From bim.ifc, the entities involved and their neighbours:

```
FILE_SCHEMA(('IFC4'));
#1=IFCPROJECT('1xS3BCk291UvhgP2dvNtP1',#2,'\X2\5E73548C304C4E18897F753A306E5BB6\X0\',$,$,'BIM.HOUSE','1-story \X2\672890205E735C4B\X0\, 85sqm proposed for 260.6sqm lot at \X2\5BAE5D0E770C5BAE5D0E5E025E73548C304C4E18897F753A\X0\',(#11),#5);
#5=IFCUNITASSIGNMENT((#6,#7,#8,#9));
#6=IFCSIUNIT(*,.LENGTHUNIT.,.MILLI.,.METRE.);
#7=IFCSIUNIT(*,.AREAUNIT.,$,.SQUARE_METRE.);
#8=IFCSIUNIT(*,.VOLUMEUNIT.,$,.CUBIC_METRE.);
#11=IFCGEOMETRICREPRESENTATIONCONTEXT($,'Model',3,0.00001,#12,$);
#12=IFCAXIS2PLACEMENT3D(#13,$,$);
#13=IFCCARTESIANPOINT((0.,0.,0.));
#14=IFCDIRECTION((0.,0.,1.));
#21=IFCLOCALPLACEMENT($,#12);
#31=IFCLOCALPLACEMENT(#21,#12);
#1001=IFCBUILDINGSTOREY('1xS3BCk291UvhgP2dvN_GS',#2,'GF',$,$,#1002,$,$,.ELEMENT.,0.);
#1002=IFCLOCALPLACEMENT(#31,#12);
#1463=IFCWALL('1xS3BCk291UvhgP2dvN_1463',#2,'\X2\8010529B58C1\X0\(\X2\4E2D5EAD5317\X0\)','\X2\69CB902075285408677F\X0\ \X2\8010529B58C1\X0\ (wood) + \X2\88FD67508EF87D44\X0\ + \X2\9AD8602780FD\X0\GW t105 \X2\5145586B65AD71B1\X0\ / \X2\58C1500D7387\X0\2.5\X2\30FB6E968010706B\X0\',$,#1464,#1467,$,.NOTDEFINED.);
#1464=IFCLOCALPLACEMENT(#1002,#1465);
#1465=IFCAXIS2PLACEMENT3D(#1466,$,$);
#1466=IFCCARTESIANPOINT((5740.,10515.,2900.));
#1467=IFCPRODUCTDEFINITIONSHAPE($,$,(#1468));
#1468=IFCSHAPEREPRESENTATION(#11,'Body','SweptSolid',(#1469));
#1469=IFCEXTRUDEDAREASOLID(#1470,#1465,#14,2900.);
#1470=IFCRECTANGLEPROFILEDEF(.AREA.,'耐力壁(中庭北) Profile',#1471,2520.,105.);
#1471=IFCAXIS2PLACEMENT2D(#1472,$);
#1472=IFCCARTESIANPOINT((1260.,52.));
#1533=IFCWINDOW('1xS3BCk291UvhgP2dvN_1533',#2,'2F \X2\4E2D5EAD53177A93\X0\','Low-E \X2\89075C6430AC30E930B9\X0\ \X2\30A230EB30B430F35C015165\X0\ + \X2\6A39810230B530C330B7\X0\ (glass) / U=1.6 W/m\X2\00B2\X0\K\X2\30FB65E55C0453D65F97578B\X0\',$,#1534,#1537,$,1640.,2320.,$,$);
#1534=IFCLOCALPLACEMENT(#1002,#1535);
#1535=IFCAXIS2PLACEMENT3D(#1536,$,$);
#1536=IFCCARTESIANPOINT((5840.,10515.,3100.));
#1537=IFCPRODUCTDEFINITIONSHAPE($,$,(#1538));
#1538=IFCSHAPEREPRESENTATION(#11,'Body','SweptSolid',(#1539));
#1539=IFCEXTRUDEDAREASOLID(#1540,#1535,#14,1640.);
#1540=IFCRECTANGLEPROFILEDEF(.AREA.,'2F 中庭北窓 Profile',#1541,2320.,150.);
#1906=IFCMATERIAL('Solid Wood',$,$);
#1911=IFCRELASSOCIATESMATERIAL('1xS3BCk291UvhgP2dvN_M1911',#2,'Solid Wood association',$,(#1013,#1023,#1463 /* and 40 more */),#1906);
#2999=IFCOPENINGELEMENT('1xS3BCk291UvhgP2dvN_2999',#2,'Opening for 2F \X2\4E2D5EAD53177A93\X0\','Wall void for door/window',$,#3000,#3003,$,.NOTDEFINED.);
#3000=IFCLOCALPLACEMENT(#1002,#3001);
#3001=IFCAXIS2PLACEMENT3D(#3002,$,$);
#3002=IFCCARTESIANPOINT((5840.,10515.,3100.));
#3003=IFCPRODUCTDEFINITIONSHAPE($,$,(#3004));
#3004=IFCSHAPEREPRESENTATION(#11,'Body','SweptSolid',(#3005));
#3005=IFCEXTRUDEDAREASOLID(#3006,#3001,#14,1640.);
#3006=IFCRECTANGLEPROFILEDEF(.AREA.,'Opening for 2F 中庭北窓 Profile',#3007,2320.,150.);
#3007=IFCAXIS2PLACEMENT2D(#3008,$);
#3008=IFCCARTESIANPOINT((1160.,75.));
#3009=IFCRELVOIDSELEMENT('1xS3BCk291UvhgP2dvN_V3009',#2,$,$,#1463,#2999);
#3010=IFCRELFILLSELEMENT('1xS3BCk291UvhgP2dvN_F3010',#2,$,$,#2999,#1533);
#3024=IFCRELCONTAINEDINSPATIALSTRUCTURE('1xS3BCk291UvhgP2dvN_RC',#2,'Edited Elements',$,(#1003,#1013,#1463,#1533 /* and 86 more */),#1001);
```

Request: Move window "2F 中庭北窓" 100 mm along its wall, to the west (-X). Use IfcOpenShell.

```python
import ifcopenshell
import ifcopenshell.api.geometry
import ifcopenshell.util.placement
import ifcopenshell.util.unit

model = ifcopenshell.open("bim.ifc")
unit_scale = ifcopenshell.util.unit.calculate_unit_scale(model)

window = model.by_guid("1xS3BCk291UvhgP2dvN_1533")
opening = window.FillsVoids[0].RelatingOpeningElement
wall = opening.VoidsElements[0].RelatingBuildingElement

wall_matrix = ifcopenshell.util.placement.get_local_placement(wall.ObjectPlacement)
shift = wall_matrix[:3, 0] * -0.1 / unit_scale
before = ifcopenshell.util.placement.get_local_placement(window.ObjectPlacement)[:3, 3].copy()

# The window is not placed relative to its opening, so move both.
for product in (opening, window):
    matrix = ifcopenshell.util.placement.get_local_placement(product.ObjectPlacement)
    matrix[:3, 3] += shift
    ifcopenshell.api.geometry.edit_object_placement(model, product=product, matrix=matrix, is_si=False)

after = ifcopenshell.util.placement.get_local_placement(window.ObjectPlacement)[:3, 3]
print("window moved by", (after - before).round(3) + 0.0)

model.write("bim-out.ifc")
```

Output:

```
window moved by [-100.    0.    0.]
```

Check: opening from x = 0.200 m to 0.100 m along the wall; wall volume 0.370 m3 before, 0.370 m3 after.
